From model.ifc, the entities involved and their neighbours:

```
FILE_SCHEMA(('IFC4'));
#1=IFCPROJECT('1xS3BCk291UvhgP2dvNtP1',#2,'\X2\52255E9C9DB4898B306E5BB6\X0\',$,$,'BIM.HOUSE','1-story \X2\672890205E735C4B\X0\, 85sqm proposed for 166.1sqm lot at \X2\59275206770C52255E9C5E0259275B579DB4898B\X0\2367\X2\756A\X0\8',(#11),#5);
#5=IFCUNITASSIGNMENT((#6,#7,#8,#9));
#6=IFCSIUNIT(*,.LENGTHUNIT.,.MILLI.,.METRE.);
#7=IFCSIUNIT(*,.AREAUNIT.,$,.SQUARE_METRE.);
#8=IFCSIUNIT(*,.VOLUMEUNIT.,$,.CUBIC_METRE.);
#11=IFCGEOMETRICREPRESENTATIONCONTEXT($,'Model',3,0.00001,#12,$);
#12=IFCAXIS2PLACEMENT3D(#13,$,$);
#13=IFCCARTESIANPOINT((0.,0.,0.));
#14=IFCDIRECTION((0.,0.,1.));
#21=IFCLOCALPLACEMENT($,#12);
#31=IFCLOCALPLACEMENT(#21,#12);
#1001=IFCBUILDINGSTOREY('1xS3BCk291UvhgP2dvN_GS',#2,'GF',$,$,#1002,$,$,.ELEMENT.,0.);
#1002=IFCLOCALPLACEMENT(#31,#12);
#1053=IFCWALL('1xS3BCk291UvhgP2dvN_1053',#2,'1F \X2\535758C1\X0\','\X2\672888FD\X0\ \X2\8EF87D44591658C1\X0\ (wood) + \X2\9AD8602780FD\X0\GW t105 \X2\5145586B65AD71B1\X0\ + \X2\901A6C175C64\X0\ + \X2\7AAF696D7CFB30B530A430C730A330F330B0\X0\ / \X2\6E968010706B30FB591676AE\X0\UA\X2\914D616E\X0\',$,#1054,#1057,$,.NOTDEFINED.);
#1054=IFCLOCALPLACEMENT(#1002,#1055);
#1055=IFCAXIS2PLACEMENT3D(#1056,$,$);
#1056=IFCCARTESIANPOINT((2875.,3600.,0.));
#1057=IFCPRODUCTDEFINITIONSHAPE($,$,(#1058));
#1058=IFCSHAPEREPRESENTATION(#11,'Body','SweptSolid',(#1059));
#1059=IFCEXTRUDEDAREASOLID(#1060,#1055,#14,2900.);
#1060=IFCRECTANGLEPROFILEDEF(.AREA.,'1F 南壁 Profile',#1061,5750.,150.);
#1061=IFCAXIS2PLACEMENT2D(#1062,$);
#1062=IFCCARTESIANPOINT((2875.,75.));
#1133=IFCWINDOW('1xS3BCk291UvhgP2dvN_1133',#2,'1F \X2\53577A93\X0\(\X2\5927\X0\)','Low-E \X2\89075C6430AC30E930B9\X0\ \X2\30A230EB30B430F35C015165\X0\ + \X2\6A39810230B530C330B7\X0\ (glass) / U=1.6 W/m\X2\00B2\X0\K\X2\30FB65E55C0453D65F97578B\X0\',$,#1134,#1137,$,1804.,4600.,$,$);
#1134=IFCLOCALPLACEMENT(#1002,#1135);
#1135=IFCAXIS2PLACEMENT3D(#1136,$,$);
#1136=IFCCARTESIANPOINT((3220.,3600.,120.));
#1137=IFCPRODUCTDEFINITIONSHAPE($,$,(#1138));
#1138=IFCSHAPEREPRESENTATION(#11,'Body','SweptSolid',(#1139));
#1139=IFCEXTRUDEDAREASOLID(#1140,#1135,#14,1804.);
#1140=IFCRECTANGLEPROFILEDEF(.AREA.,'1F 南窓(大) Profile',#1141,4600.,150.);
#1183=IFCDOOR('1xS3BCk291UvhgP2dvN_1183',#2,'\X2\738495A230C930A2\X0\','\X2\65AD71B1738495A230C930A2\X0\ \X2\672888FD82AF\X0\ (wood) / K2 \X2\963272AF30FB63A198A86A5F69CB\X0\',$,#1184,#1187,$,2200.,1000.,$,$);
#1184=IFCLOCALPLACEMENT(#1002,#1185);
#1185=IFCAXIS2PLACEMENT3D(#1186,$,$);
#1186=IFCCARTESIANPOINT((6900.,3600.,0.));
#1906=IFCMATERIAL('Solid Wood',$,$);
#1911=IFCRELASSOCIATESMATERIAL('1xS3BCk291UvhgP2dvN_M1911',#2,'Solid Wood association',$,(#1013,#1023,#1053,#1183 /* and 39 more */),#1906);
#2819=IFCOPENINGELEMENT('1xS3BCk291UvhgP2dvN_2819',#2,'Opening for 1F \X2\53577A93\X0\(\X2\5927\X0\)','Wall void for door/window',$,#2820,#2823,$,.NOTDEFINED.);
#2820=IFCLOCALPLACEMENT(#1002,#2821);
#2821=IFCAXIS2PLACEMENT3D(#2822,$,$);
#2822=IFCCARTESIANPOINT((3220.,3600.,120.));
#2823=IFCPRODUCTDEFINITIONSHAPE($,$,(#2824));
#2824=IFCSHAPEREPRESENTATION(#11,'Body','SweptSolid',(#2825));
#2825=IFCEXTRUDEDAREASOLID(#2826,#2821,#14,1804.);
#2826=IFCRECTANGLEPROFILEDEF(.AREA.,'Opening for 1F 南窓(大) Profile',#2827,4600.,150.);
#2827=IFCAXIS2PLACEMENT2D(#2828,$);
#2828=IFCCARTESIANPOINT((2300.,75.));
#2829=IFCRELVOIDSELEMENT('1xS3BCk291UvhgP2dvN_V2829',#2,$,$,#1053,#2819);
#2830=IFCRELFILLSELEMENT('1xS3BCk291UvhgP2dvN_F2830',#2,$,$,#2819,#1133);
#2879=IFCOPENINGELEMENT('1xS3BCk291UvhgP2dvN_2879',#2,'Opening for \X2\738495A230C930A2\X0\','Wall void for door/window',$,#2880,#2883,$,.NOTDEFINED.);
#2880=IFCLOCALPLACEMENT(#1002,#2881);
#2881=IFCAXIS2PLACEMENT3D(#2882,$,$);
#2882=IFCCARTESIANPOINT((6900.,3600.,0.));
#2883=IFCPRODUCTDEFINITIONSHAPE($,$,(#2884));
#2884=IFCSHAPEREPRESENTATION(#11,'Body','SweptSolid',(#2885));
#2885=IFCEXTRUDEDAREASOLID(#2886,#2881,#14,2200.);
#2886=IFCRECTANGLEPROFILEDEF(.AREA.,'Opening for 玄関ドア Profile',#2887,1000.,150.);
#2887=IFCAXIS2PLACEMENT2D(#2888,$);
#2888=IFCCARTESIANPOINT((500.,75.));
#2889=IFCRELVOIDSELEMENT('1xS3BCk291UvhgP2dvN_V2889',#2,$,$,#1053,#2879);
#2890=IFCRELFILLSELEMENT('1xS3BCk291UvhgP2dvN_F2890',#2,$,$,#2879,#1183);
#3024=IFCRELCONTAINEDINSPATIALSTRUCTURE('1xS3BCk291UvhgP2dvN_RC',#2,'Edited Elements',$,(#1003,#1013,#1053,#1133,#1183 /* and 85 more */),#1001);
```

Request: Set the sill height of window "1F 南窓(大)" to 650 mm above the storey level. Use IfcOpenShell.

```python
import numpy as np
import ifcopenshell
import ifcopenshell.api.geometry
import ifcopenshell.geom
import ifcopenshell.util.element
import ifcopenshell.util.placement
import ifcopenshell.util.shape
import ifcopenshell.util.unit

model = ifcopenshell.open("model.ifc")
unit_scale = ifcopenshell.util.unit.calculate_unit_scale(model)

window = model.by_guid("1xS3BCk291UvhgP2dvN_1133")
opening = window.FillsVoids[0].RelatingOpeningElement
storey = ifcopenshell.util.element.get_container(window, ifc_class="IfcBuildingStorey")
level = ifcopenshell.util.placement.get_local_placement(storey.ObjectPlacement)[2, 3]

# The opening's origin need not be at the sill, so measure its lowest point.
shape = ifcopenshell.geom.create_shape(ifcopenshell.geom.settings(), opening)
bottom = ifcopenshell.util.shape.get_shape_bottom_elevation(shape, shape.geometry) / unit_scale
dz = level + 0.65 / unit_scale - bottom

shift = np.array([0.0, 0.0, dz])
# The window is not placed relative to its opening, so move both.
for product in (opening, window):
    matrix = ifcopenshell.util.placement.get_local_placement(product.ObjectPlacement)
    matrix[:3, 3] += shift
    ifcopenshell.api.geometry.edit_object_placement(model, product=product, matrix=matrix, is_si=False)

print(f"moved by {dz * unit_scale:+.3f} m")

model.write("model_updated.ifc")
```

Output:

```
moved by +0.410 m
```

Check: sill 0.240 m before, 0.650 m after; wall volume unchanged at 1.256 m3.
